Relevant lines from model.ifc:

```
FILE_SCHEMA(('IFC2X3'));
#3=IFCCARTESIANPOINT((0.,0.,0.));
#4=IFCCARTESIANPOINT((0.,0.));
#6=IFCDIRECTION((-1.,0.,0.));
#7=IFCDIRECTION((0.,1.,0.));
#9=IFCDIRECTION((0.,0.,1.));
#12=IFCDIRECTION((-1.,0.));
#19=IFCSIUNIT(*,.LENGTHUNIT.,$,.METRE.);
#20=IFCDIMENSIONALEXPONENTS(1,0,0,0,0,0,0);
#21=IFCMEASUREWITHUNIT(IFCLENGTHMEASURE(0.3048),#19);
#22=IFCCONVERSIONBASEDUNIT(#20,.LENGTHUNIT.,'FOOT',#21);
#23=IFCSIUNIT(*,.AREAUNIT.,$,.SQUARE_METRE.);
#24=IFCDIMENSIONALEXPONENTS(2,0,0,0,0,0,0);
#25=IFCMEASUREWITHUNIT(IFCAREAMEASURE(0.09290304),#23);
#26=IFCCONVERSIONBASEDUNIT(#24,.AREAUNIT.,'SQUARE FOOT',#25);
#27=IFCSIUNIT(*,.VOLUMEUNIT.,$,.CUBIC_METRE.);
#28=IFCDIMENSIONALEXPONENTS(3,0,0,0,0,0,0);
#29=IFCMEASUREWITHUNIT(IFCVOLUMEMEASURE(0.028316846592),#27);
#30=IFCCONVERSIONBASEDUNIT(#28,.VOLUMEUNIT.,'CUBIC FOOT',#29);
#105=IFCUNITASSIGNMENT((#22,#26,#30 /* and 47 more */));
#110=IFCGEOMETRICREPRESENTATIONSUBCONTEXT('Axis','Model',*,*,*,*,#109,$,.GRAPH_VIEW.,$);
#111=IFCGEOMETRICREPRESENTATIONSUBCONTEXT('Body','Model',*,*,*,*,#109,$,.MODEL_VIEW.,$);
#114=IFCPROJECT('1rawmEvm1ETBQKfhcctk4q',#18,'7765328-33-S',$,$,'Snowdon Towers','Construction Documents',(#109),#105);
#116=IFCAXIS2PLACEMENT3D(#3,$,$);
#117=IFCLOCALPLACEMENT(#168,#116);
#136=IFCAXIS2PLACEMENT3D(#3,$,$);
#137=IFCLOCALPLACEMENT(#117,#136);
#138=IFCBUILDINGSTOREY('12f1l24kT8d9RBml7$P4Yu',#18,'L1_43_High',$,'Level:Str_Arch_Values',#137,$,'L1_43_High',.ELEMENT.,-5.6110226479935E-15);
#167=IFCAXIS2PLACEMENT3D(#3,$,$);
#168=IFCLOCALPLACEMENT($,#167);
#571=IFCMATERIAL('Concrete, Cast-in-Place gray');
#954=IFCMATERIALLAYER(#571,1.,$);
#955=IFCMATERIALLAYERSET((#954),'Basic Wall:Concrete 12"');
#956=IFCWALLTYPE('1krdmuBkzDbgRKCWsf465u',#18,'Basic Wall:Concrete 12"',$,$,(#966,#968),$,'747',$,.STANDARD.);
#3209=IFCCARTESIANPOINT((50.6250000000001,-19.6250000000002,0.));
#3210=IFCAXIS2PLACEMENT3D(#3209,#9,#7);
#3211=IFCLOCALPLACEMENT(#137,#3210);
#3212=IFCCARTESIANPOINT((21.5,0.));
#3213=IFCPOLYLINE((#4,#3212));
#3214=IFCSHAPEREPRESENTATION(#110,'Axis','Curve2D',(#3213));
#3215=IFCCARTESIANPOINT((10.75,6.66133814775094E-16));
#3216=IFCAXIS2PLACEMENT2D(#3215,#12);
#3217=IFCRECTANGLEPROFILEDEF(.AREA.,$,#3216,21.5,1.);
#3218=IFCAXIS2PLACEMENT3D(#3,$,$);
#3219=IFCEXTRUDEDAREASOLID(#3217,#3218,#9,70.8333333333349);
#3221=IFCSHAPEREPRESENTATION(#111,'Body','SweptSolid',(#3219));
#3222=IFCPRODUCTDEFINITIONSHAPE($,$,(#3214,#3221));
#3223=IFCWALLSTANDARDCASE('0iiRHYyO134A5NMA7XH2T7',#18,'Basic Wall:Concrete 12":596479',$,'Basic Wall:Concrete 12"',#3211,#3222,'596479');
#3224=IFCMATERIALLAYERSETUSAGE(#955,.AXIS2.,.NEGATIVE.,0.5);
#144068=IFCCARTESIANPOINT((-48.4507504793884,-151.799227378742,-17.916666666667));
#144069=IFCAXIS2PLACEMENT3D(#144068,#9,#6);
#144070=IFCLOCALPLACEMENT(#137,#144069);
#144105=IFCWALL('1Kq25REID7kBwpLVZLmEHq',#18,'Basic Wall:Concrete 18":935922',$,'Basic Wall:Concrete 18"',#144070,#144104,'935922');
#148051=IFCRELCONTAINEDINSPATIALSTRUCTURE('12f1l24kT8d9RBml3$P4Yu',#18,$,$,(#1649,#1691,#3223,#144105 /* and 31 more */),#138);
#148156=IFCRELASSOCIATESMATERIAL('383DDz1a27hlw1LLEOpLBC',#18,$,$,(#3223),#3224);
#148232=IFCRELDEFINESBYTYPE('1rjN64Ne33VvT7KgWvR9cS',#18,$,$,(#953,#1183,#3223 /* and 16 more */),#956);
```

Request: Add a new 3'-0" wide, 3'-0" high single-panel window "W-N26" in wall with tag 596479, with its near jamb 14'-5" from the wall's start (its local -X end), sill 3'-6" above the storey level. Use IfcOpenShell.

```python
import numpy as np
import ifcopenshell
import ifcopenshell.api.feature
import ifcopenshell.api.geometry
import ifcopenshell.api.root
import ifcopenshell.api.spatial
import ifcopenshell.api.type
import ifcopenshell.geom
import ifcopenshell.util.element
import ifcopenshell.util.placement
import ifcopenshell.util.representation
import ifcopenshell.util.shape
import ifcopenshell.util.unit

model = ifcopenshell.open("model.ifc")
unit_scale = ifcopenshell.util.unit.calculate_unit_scale(model)
settings = ifcopenshell.geom.settings()


def volume(element):
    """Net volume in cubic metres, openings subtracted."""
    shape = ifcopenshell.geom.create_shape(settings, element)
    return ifcopenshell.util.shape.get_volume(shape.geometry)


wall = model.by_id(3223)
storey = ifcopenshell.util.element.get_container(wall, ifc_class="IfcBuildingStorey")
context = ifcopenshell.util.representation.get_context(model, "Model", "Body", "MODEL_VIEW")
before = volume(wall)

width, height, from_end, sill = 0.9144, 0.9144, 4.3942, 1.0668  # metres

# The wall runs along its own X axis, and the end named is its -X end.
wall_shape = ifcopenshell.geom.create_shape(settings, wall)
x, y, z = ifcopenshell.util.shape.get_vertices(wall_shape.geometry).T
start = x.min() + from_end
face, thickness = float(y.min()), float(y.max() - y.min())
wall_matrix = ifcopenshell.util.placement.get_local_placement(wall.ObjectPlacement)
level = ifcopenshell.util.placement.get_local_placement(storey.ObjectPlacement)[2, 3]


def in_wall(x, y):
    """Placement at x, y metres in the wall's axes, at sill height."""
    matrix = wall_matrix.copy()
    matrix[:, 3] = wall_matrix @ np.array([x / unit_scale, y / unit_scale, 0.0, 1.0])
    matrix[2, 3] = level + sill / unit_scale
    return matrix


# Opening: a box that overshoots both wall faces by 50 mm.
opening = ifcopenshell.api.root.create_entity(model, ifc_class="IfcOpeningElement")
box = ifcopenshell.api.geometry.add_wall_representation(
    model, context=context, length=width, height=height, thickness=thickness + 0.1
)
ifcopenshell.api.geometry.assign_representation(model, product=opening, representation=box)
ifcopenshell.api.geometry.edit_object_placement(model, product=opening, matrix=in_wall(start, face - 0.05), is_si=False)
ifcopenshell.api.feature.add_feature(model, feature=opening, element=wall)

window = ifcopenshell.api.root.create_entity(model, ifc_class="IfcWindow", name="W-N26")
window.OverallWidth, window.OverallHeight = width / unit_scale, height / unit_scale
body = ifcopenshell.api.geometry.add_window_representation(
    model,
    context=context,
    overall_width=window.OverallWidth,
    overall_height=window.OverallHeight,
    partition_type="SINGLE_PANEL",
)
ifcopenshell.api.geometry.assign_representation(model, product=window, representation=body)
ifcopenshell.api.spatial.assign_container(model, products=[window], relating_structure=storey)
fills = ifcopenshell.api.feature.add_filling(model, opening=opening, element=window)
fills.OwnerHistory = window.OwnerHistory  # required in IFC2X3

# IFC2X3 keeps the operation on the window style.
style = ifcopenshell.api.root.create_entity(model, ifc_class="IfcWindowStyle", name="W-N26")
style.OperationType, style.ConstructionType = "SINGLE_PANEL", "NOTDEFINED"
style.ParameterTakesPrecedence = style.Sizeable = False
ifcopenshell.api.type.assign_type(model, related_objects=[window], relating_type=style)

# Centre the window in the wall's thickness.
ifcopenshell.api.geometry.edit_object_placement(model, product=window, matrix=in_wall(start, face), is_si=False)
window_shape = ifcopenshell.geom.create_shape(settings, window)
depth = ifcopenshell.util.shape.get_vertices(window_shape.geometry)[:, 1]
offset = face + thickness / 2 - (depth.min() + depth.max()) / 2
ifcopenshell.api.geometry.edit_object_placement(model, product=window, matrix=in_wall(start, offset), is_si=False)

after = volume(wall)

print(f"wall volume {before:.3f} -> {after:.3f} m3")

model.write("model-out.ifc")
```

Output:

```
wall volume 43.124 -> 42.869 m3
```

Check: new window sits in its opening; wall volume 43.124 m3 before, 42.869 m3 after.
